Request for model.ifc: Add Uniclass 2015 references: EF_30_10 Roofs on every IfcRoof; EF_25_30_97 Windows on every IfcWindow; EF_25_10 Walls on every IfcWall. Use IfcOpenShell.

First a look at what the model holds.

```python
import ifcopenshell

model = ifcopenshell.open("model.ifc")
print(model.schema)
print("classifications:", [c.Name for c in model.by_type("IfcClassification")])
for ifc_class in ("IfcDoor", "IfcRoof", "IfcStair", "IfcWall", "IfcWindow"):
    print(ifc_class, len(model.by_type(ifc_class)))
```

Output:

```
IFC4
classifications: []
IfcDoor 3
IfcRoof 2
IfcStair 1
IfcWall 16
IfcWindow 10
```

```python
import ifcopenshell
import ifcopenshell.api.classification

model = ifcopenshell.open("model.ifc")

system = ifcopenshell.api.classification.add_classification(model, classification="Uniclass 2015")

codes = {
    "IfcRoof": ("EF_30_10", "Roofs"),
    "IfcWindow": ("EF_25_30_97", "Windows"),
    "IfcWall": ("EF_25_10", "Walls"),
}
for ifc_class, (code, name) in codes.items():
    products = model.by_type(ifc_class)
    ifcopenshell.api.classification.add_reference(
        model, products=products, classification=system, identification=code, name=name
    )
    print(code, len(products))

model.write("model_edited.ifc")
```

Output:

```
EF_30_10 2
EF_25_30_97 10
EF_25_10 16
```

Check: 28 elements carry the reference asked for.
